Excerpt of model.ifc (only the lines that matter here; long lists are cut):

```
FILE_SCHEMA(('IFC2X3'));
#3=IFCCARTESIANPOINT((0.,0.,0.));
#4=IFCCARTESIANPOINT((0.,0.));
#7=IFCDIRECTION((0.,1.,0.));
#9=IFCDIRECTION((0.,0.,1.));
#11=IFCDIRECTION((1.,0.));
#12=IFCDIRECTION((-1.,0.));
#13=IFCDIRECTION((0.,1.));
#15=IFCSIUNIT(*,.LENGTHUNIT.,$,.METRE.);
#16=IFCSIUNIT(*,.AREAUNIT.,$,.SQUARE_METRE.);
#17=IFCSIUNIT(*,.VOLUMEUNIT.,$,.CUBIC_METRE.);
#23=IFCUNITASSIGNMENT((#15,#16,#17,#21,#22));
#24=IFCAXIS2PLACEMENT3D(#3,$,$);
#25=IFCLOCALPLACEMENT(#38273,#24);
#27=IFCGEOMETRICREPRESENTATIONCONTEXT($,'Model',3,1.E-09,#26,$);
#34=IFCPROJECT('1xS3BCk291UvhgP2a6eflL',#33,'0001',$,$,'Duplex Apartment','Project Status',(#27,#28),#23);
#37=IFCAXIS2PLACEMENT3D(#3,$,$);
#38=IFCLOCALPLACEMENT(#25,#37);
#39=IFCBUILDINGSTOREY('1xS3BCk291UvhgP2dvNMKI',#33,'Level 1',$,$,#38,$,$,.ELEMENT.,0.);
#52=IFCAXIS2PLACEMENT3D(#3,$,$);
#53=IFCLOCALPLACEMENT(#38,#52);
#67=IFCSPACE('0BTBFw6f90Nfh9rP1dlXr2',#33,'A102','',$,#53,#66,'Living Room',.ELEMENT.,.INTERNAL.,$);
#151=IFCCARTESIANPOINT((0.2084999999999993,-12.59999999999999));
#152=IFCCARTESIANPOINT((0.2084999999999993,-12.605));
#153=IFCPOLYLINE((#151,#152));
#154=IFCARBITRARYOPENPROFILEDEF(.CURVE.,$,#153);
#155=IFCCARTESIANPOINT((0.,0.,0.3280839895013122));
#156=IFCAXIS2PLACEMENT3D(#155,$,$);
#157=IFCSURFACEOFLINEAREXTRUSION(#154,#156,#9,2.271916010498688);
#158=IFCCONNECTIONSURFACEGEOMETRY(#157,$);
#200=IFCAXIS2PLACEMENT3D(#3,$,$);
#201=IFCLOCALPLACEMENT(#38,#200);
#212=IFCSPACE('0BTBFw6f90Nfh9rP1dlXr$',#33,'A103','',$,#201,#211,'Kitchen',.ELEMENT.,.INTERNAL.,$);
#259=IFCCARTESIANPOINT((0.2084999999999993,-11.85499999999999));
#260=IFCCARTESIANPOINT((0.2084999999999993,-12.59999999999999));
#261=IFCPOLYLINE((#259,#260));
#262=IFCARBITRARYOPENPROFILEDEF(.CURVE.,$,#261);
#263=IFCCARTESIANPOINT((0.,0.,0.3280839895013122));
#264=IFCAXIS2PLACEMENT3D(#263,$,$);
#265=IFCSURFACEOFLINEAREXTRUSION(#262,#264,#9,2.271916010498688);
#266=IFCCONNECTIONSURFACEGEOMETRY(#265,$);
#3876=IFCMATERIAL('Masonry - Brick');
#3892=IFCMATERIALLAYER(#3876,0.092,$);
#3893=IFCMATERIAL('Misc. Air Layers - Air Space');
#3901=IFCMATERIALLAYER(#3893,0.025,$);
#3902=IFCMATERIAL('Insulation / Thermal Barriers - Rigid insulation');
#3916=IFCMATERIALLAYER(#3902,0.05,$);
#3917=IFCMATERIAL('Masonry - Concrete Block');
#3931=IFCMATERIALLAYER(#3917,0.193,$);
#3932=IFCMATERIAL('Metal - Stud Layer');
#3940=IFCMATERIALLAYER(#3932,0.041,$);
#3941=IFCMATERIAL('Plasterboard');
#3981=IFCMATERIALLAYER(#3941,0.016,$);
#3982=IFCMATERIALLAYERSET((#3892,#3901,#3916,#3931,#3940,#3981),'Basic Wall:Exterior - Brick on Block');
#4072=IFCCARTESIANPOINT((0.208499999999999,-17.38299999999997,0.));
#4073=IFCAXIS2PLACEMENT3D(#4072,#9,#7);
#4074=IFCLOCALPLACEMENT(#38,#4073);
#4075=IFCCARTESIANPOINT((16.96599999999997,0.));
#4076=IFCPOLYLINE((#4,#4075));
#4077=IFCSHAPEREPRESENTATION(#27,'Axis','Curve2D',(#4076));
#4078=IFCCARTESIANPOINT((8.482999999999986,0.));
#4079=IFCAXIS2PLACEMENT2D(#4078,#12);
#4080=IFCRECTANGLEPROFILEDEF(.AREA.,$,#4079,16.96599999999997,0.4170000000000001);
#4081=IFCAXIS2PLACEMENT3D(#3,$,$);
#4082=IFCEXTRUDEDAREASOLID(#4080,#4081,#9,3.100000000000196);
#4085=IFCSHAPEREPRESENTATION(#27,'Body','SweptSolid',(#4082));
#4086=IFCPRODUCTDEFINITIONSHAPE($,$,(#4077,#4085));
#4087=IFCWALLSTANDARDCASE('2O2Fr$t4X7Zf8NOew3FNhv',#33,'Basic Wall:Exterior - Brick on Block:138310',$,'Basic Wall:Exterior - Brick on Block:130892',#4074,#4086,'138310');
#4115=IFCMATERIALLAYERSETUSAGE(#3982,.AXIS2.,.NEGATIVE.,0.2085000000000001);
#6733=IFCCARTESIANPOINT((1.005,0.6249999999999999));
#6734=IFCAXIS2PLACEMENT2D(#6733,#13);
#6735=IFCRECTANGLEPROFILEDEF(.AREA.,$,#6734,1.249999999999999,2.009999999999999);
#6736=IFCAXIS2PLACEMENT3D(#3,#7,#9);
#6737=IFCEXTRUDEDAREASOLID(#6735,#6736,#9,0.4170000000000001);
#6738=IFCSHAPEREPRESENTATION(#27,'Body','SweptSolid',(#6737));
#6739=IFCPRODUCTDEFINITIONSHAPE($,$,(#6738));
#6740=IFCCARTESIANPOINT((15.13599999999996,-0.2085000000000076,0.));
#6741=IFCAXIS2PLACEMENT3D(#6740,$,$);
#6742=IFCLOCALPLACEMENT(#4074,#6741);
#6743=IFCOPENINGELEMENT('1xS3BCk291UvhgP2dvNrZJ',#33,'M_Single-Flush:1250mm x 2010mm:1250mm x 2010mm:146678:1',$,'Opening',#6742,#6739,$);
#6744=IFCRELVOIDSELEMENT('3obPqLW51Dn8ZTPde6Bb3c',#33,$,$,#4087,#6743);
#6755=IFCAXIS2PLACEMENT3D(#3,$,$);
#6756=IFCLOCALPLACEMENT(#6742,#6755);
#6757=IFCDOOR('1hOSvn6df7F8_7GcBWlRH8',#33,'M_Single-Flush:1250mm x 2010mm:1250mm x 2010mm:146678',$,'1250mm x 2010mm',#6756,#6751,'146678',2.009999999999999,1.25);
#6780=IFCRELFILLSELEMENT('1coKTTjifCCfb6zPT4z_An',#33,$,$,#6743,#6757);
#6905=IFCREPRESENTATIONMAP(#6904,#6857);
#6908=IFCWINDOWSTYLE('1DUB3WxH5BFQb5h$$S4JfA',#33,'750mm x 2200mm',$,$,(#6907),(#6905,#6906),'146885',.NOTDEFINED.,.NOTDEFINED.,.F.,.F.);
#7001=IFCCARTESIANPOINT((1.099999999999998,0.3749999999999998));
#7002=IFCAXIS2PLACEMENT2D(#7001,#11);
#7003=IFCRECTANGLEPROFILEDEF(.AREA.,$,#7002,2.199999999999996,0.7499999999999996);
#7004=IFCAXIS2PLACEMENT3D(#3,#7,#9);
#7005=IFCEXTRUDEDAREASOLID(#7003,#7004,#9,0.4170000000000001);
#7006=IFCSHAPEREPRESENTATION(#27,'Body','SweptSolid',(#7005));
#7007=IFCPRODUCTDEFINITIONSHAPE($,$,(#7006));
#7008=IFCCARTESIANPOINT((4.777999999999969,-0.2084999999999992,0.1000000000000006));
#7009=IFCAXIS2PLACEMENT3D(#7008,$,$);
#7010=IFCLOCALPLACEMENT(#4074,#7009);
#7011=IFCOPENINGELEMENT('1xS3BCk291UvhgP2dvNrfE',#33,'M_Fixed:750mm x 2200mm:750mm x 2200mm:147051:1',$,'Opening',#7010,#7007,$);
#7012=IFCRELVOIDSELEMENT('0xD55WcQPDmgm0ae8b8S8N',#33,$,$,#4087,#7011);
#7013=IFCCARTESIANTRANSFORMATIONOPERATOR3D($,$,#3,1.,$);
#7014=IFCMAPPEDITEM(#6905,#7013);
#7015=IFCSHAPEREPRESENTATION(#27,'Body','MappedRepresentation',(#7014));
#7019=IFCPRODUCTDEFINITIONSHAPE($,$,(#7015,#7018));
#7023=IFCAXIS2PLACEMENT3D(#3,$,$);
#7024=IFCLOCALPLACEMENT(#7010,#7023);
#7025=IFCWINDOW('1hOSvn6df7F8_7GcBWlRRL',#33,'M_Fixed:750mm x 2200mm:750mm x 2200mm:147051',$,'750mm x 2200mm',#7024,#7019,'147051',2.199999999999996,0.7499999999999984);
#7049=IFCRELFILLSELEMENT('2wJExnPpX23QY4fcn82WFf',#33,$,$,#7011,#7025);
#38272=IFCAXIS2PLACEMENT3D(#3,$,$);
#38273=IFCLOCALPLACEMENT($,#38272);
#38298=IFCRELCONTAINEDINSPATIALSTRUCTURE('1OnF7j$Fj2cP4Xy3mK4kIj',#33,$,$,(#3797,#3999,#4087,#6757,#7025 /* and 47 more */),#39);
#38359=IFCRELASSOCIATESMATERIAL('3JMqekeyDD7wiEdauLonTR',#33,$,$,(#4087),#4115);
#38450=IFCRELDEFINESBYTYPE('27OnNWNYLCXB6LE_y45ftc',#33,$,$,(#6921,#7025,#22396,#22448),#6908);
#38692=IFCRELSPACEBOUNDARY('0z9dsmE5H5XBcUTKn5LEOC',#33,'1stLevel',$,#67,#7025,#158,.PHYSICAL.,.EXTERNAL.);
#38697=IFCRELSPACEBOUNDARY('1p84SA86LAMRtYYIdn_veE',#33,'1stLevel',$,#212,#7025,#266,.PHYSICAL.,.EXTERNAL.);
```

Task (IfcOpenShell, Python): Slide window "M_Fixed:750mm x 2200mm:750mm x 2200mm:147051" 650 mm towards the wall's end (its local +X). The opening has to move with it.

```python
import numpy as np
import ifcopenshell
import ifcopenshell.api.geometry
import ifcopenshell.util.placement

model = ifcopenshell.open("model.ifc")

window = model.by_guid("1hOSvn6df7F8_7GcBWlRRL")
opening = window.FillsVoids[0].RelatingOpeningElement
wall = opening.VoidsElements[0].RelatingBuildingElement

wall_matrix = ifcopenshell.util.placement.get_local_placement(wall.ObjectPlacement)
shift = wall_matrix[:3, 0] * 0.65
before = ifcopenshell.util.placement.get_local_placement(window.ObjectPlacement)[:3, 3].copy()

# The window is placed relative to its opening, so it follows when the opening moves.
matrix = ifcopenshell.util.placement.get_local_placement(opening.ObjectPlacement)
matrix[:3, 3] += shift
ifcopenshell.api.geometry.edit_object_placement(
    model, product=opening, matrix=matrix, is_si=False, should_transform_children=True
)

# Space boundary surfaces are stored in each space's coordinates; move them too.
for rel in window.ProvidesBoundaries:
    if not rel.ConnectionGeometry:
        continue
    surface = rel.ConnectionGeometry.SurfaceOnRelatingElement
    space_matrix = ifcopenshell.util.placement.get_local_placement(rel.RelatingSpace.ObjectPlacement)
    point = np.array(surface.Position.Location.Coordinates) + space_matrix[:3, :3].T @ shift
    surface.Position = model.createIfcAxis2Placement3D(
        model.createIfcCartesianPoint(point.tolist()), surface.Position.Axis, surface.Position.RefDirection
    )

after = ifcopenshell.util.placement.get_local_placement(window.ObjectPlacement)[:3, 3]
print("window moved by", (after - before).round(3) + 0.0)

model.write("model_updated.ifc")
```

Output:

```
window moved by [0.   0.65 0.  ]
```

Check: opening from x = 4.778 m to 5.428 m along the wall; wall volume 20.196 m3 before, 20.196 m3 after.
